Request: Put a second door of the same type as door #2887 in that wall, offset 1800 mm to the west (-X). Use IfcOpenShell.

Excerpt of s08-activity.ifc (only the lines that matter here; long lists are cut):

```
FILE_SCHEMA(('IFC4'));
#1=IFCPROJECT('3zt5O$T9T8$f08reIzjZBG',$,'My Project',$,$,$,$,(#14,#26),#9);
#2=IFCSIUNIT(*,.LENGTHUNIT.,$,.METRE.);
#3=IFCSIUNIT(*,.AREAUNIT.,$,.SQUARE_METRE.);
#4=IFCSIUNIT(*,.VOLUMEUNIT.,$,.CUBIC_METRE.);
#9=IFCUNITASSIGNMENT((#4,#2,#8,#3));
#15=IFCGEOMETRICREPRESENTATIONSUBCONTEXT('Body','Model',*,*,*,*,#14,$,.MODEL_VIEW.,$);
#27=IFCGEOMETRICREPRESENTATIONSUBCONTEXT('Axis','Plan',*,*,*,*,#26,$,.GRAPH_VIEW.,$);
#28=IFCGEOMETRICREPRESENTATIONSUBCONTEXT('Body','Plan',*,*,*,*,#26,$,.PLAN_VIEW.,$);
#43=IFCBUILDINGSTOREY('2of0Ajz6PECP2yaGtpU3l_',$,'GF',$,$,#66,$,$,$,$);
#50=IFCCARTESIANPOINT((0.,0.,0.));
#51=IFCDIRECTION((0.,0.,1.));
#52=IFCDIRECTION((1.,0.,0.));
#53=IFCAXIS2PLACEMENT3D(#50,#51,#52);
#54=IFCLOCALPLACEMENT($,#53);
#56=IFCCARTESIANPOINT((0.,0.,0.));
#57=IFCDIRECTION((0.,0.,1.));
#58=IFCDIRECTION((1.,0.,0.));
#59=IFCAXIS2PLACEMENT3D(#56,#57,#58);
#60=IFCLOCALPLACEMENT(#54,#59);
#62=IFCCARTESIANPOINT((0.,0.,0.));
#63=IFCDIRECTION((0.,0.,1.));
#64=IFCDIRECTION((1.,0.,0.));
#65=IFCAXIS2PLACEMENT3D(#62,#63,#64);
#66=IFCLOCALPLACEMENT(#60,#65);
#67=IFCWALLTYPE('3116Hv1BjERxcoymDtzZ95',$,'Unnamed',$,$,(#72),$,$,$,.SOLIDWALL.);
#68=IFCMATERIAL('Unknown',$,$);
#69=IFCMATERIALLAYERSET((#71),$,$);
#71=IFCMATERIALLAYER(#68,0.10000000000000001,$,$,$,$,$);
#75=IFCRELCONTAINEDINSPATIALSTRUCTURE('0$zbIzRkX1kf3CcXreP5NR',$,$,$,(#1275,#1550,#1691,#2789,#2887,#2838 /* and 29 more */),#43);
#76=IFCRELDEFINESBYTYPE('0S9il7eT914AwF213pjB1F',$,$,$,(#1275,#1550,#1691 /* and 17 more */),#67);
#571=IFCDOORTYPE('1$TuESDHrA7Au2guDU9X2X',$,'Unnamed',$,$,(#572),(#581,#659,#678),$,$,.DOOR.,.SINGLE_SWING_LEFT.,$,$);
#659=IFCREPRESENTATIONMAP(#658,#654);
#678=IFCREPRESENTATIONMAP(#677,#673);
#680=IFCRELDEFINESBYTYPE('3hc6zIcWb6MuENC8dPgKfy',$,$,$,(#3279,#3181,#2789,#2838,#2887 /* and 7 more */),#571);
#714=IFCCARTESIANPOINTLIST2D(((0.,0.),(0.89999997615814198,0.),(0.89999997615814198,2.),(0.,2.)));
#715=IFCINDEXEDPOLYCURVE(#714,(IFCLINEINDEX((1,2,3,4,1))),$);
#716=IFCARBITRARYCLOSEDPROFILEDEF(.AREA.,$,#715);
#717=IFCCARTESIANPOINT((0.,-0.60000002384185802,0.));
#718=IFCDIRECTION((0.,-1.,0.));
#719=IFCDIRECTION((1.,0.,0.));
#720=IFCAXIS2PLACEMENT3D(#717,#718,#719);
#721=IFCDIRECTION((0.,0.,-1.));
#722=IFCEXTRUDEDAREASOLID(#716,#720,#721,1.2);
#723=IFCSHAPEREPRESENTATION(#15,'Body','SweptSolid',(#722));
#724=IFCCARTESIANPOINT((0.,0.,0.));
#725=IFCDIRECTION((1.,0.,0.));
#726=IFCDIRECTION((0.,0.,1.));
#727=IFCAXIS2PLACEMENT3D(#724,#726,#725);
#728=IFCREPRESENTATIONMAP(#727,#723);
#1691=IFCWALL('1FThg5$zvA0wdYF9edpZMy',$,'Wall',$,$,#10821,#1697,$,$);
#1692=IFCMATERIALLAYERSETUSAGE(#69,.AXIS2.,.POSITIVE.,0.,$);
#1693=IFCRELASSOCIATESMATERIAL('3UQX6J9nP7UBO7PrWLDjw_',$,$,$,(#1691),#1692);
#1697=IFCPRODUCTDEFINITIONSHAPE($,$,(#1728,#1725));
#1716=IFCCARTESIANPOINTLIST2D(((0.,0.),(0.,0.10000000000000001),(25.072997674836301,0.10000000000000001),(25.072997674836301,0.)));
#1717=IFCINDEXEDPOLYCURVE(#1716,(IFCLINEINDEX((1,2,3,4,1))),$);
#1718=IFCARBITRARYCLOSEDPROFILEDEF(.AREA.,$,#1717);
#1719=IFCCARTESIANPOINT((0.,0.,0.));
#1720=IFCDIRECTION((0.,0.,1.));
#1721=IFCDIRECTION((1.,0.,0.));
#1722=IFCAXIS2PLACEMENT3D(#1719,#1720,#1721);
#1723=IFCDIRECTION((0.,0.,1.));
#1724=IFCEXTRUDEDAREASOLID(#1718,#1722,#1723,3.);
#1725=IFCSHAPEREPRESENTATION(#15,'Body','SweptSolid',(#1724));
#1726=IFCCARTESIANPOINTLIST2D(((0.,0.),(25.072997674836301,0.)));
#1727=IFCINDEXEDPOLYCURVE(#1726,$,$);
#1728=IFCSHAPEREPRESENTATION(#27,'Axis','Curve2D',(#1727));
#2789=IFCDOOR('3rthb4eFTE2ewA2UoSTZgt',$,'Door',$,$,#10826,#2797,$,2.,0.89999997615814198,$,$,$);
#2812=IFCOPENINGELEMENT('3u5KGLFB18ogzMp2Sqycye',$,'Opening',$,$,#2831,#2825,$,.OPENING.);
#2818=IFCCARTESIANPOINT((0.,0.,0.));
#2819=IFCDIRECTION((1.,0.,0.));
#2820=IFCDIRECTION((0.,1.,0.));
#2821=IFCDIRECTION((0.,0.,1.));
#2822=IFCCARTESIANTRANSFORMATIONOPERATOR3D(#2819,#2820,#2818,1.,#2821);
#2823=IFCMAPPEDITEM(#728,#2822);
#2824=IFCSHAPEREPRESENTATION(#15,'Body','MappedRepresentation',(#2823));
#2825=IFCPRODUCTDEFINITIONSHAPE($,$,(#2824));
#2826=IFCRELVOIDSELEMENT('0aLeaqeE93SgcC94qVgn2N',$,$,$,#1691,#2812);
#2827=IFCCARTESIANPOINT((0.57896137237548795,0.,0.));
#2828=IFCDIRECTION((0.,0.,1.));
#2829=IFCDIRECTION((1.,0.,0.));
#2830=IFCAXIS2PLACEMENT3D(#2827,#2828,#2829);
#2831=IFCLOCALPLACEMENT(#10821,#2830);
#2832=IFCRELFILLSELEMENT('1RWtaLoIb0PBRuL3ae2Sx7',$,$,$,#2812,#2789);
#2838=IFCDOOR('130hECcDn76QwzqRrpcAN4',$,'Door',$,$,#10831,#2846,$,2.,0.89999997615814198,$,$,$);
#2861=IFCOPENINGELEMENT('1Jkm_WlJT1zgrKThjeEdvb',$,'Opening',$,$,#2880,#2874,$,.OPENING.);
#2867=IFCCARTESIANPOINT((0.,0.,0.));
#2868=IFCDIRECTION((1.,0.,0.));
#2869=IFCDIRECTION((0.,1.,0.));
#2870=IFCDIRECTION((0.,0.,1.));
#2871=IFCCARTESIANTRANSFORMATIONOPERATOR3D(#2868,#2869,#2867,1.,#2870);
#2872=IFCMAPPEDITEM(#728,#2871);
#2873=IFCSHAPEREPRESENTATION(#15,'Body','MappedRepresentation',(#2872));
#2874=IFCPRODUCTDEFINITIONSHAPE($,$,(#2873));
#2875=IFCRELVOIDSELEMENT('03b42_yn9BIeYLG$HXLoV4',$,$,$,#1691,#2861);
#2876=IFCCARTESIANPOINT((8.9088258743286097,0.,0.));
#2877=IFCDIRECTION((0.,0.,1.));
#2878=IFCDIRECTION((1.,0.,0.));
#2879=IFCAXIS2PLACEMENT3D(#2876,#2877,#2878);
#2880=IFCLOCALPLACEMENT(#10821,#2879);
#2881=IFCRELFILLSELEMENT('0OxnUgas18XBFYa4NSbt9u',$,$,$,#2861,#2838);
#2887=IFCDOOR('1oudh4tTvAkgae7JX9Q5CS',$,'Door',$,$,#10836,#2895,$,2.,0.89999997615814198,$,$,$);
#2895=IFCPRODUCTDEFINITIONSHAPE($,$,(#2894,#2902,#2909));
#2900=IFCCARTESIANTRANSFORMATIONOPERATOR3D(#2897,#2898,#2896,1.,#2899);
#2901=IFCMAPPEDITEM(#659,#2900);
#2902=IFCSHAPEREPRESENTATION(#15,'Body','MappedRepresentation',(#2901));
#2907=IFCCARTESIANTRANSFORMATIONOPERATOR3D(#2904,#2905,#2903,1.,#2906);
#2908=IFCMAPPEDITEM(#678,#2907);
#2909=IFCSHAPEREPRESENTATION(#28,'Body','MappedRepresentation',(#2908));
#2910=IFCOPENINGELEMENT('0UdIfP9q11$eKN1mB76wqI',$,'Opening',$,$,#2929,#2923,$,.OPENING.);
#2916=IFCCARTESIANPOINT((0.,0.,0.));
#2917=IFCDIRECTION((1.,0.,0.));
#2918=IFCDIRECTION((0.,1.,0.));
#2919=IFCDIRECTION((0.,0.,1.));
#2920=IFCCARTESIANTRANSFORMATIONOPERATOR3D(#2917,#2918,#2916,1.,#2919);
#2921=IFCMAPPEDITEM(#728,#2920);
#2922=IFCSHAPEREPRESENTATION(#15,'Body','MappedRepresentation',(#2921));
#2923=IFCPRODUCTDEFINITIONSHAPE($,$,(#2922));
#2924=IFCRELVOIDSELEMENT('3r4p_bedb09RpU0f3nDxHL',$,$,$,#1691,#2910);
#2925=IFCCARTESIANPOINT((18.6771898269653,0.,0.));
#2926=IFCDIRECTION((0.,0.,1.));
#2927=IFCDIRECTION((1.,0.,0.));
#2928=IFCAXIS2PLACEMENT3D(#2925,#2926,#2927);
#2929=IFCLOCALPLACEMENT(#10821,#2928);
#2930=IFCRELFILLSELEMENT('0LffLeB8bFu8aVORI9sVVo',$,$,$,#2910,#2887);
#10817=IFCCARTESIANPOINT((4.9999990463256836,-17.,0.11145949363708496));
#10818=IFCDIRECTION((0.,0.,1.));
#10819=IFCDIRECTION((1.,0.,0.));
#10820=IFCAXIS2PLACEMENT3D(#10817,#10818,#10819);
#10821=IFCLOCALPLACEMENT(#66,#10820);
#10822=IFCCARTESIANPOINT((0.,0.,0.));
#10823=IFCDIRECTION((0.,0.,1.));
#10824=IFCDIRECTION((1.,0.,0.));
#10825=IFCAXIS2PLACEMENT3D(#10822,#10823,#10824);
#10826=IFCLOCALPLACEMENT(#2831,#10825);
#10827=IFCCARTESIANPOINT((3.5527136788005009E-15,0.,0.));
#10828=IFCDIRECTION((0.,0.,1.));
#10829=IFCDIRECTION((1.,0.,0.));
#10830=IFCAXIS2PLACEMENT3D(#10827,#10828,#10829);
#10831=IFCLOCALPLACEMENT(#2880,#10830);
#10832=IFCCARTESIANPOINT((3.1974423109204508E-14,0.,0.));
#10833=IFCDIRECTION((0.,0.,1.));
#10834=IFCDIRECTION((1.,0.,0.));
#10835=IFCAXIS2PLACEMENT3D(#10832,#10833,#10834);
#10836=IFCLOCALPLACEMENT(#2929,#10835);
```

```python
import ifcopenshell
import ifcopenshell.api.feature
import ifcopenshell.api.geometry
import ifcopenshell.api.root
import ifcopenshell.geom
import ifcopenshell.util.element
import ifcopenshell.util.placement
import ifcopenshell.util.shape
import ifcopenshell.util.unit

model = ifcopenshell.open("s08-activity.ifc")
unit_scale = ifcopenshell.util.unit.calculate_unit_scale(model)
settings = ifcopenshell.geom.settings()


def volume(element):
    """Net volume in cubic metres, openings subtracted."""
    shape = ifcopenshell.geom.create_shape(settings, element)
    return ifcopenshell.util.shape.get_volume(shape.geometry)


door = model.by_guid("1oudh4tTvAkgae7JX9Q5CS")
opening = door.FillsVoids[0].RelatingOpeningElement
wall = opening.VoidsElements[0].RelatingBuildingElement
before = volume(wall)
shift = ifcopenshell.util.placement.get_local_placement(wall.ObjectPlacement)[:3, 0] * -1.8 / unit_scale

# copy_class copies the void relationship, type, container and properties, but no geometry.
new_opening = ifcopenshell.api.root.copy_class(model, product=opening)
new_opening.Representation = ifcopenshell.util.element.copy_deep(
    model, opening.Representation, exclude=["IfcGeometricRepresentationContext", "IfcRepresentationMap"]
)
new_door = ifcopenshell.api.root.copy_class(model, product=door)
new_door.Representation = ifcopenshell.util.element.copy_deep(
    model, door.Representation, exclude=["IfcGeometricRepresentationContext", "IfcRepresentationMap"]
)
ifcopenshell.api.feature.add_filling(model, opening=new_opening, element=new_door)

for old, new in ((opening, new_opening), (door, new_door)):
    matrix = ifcopenshell.util.placement.get_local_placement(old.ObjectPlacement)
    matrix[:3, 3] += shift
    ifcopenshell.api.geometry.edit_object_placement(model, product=new, matrix=matrix, is_si=False)

after = volume(wall)

print(f"wall volume {before:.3f} -> {after:.3f} m3")

model.write("s08-activity_edited.ifc")
```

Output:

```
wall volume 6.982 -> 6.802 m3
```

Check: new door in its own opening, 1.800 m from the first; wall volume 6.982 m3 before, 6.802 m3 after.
